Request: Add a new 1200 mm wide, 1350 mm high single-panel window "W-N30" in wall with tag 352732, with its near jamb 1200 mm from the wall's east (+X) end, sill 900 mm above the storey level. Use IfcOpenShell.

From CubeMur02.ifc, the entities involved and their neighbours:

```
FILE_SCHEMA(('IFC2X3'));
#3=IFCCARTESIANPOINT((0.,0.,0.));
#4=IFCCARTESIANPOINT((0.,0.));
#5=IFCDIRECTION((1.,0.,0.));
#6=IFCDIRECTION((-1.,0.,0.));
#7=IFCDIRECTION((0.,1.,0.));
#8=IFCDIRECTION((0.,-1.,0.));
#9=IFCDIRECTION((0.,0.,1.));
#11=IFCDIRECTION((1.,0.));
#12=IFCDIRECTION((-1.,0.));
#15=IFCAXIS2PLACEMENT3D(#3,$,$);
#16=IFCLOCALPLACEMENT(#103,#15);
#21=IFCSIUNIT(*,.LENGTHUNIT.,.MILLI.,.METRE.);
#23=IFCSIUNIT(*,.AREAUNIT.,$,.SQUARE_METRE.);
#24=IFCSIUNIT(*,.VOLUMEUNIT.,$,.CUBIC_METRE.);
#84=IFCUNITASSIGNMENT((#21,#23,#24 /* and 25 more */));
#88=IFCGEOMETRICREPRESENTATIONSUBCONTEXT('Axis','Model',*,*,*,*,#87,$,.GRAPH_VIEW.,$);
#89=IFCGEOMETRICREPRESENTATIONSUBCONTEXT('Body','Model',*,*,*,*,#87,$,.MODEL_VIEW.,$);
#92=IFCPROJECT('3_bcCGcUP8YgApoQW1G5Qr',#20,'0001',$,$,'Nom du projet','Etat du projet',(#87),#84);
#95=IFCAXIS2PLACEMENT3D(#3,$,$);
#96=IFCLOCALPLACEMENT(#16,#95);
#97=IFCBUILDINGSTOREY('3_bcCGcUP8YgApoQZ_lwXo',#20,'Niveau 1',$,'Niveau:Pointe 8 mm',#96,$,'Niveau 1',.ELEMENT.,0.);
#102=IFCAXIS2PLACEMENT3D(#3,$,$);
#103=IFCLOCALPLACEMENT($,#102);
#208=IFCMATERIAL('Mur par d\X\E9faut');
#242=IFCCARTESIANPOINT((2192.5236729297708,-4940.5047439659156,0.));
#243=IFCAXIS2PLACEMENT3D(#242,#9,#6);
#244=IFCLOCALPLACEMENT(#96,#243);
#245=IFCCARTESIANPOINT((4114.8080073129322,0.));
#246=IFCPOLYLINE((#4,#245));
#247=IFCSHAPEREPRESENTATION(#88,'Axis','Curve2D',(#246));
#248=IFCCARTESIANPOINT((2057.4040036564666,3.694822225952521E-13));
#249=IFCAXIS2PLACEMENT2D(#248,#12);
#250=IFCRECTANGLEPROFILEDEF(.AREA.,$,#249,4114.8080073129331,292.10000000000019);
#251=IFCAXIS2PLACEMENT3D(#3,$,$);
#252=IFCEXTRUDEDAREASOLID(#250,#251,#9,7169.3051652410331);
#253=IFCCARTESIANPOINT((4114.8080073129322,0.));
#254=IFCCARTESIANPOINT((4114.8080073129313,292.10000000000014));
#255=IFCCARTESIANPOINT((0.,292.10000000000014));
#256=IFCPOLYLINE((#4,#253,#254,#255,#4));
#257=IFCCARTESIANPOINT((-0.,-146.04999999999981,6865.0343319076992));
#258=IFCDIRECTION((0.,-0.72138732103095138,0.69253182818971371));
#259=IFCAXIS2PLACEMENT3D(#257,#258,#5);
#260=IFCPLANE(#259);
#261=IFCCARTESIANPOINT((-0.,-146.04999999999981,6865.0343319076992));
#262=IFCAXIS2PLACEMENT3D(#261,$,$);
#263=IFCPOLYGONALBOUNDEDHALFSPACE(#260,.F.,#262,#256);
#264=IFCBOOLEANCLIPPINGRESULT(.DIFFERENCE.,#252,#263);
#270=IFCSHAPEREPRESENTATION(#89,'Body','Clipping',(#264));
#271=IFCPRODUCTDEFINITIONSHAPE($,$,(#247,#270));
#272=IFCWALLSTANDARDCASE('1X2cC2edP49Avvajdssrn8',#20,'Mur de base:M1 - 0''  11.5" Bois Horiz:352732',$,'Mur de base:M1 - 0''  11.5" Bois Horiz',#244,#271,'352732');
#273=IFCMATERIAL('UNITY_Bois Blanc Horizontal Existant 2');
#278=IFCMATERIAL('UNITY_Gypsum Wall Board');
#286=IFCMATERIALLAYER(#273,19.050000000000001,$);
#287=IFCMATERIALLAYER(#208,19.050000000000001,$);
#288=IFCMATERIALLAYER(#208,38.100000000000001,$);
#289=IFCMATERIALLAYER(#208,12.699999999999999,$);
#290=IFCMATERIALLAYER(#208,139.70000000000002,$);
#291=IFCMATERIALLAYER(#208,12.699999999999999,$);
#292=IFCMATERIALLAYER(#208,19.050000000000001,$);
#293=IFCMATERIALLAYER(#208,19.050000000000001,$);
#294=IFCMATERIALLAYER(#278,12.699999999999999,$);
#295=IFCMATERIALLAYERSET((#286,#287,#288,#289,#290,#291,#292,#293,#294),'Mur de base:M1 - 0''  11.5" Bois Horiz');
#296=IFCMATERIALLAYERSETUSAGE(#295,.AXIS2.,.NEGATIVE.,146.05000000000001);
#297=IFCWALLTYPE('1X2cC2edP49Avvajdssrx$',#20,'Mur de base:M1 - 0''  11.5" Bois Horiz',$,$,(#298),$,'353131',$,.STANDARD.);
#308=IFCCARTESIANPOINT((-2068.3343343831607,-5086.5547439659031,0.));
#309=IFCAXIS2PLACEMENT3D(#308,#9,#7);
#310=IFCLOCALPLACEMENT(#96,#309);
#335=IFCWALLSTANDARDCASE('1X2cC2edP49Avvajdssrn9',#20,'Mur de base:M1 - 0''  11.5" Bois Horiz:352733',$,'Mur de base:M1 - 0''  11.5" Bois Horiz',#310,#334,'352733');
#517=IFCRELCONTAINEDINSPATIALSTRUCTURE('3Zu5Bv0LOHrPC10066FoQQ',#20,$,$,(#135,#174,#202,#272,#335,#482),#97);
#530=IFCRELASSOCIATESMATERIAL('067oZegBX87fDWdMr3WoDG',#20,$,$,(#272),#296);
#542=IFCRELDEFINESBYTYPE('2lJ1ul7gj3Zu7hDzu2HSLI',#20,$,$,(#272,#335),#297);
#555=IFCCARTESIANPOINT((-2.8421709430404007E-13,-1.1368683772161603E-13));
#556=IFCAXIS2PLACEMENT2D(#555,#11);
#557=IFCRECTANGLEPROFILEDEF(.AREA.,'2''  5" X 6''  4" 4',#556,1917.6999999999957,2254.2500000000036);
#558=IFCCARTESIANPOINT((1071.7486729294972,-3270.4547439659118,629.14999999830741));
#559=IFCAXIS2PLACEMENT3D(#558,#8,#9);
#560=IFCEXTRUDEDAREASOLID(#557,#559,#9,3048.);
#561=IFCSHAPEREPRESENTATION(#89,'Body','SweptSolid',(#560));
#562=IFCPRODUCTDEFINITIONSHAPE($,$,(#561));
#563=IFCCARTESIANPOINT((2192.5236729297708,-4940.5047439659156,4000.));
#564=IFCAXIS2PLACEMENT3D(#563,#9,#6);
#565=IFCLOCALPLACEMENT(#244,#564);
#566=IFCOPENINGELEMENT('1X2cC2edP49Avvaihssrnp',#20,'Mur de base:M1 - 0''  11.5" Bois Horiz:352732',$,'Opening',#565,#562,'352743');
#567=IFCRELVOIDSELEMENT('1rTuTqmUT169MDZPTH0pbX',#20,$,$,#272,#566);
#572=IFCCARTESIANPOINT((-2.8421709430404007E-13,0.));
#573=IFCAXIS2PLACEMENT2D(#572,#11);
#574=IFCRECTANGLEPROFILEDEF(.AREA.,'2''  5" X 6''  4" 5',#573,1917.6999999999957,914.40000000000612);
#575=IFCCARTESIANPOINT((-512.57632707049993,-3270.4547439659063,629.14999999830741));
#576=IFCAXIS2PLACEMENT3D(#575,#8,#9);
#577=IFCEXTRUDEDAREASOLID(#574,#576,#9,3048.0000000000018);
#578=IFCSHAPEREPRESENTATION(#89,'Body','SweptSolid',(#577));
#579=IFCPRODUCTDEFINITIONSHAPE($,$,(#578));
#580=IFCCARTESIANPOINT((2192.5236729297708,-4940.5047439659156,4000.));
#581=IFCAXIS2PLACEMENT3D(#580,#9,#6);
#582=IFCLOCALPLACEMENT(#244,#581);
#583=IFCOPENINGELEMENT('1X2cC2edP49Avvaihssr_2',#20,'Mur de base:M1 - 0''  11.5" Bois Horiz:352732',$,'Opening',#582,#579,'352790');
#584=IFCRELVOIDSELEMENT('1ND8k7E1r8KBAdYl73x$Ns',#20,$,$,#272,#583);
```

```python
import numpy as np
import ifcopenshell
import ifcopenshell.api.feature
import ifcopenshell.api.geometry
import ifcopenshell.api.root
import ifcopenshell.api.spatial
import ifcopenshell.api.type
import ifcopenshell.geom
import ifcopenshell.util.element
import ifcopenshell.util.placement
import ifcopenshell.util.representation
import ifcopenshell.util.shape
import ifcopenshell.util.unit

model = ifcopenshell.open("CubeMur02.ifc")
unit_scale = ifcopenshell.util.unit.calculate_unit_scale(model)
settings = ifcopenshell.geom.settings()


def volume(element):
    """Net volume in cubic metres, openings subtracted."""
    shape = ifcopenshell.geom.create_shape(settings, element)
    return ifcopenshell.util.shape.get_volume(shape.geometry)


wall = model.by_guid("1X2cC2edP49Avvajdssrn8")
storey = ifcopenshell.util.element.get_container(wall, ifc_class="IfcBuildingStorey")
context = ifcopenshell.util.representation.get_context(model, "Model", "Body", "MODEL_VIEW")
before = volume(wall)

width, height, from_end, sill = 1.2, 1.35, 1.2, 0.9  # metres

# The wall runs along its own X axis, and the end named is its -X end.
wall_shape = ifcopenshell.geom.create_shape(settings, wall)
x, y, z = ifcopenshell.util.shape.get_vertices(wall_shape.geometry).T
start = x.min() + from_end
face, thickness = float(y.min()), float(y.max() - y.min())
wall_matrix = ifcopenshell.util.placement.get_local_placement(wall.ObjectPlacement)
level = ifcopenshell.util.placement.get_local_placement(storey.ObjectPlacement)[2, 3]


def in_wall(x, y):
    """Placement at x, y metres in the wall's axes, at sill height."""
    matrix = wall_matrix.copy()
    matrix[:, 3] = wall_matrix @ np.array([x / unit_scale, y / unit_scale, 0.0, 1.0])
    matrix[2, 3] = level + sill / unit_scale
    return matrix


# Opening: a box that overshoots both wall faces by 50 mm.
opening = ifcopenshell.api.root.create_entity(model, ifc_class="IfcOpeningElement")
box = ifcopenshell.api.geometry.add_wall_representation(
    model, context=context, length=width, height=height, thickness=thickness + 0.1
)
ifcopenshell.api.geometry.assign_representation(model, product=opening, representation=box)
ifcopenshell.api.geometry.edit_object_placement(model, product=opening, matrix=in_wall(start, face - 0.05), is_si=False)
ifcopenshell.api.feature.add_feature(model, feature=opening, element=wall)

window = ifcopenshell.api.root.create_entity(model, ifc_class="IfcWindow", name="W-N30")
window.OverallWidth, window.OverallHeight = width / unit_scale, height / unit_scale
body = ifcopenshell.api.geometry.add_window_representation(
    model,
    context=context,
    overall_width=window.OverallWidth,
    overall_height=window.OverallHeight,
    partition_type="SINGLE_PANEL",
)
ifcopenshell.api.geometry.assign_representation(model, product=window, representation=body)
ifcopenshell.api.spatial.assign_container(model, products=[window], relating_structure=storey)
fills = ifcopenshell.api.feature.add_filling(model, opening=opening, element=window)
fills.OwnerHistory = window.OwnerHistory  # required in IFC2X3

# IFC2X3 keeps the operation on the window style.
style = ifcopenshell.api.root.create_entity(model, ifc_class="IfcWindowStyle", name="W-N30")
style.OperationType, style.ConstructionType = "SINGLE_PANEL", "NOTDEFINED"
style.ParameterTakesPrecedence = style.Sizeable = False
ifcopenshell.api.type.assign_type(model, related_objects=[window], relating_type=style)

# Centre the window in the wall's thickness.
ifcopenshell.api.geometry.edit_object_placement(model, product=window, matrix=in_wall(start, face), is_si=False)
window_shape = ifcopenshell.geom.create_shape(settings, window)
depth = ifcopenshell.util.shape.get_vertices(window_shape.geometry)[:, 1]
offset = face + thickness / 2 - (depth.min() + depth.max()) / 2
ifcopenshell.api.geometry.edit_object_placement(model, product=window, matrix=in_wall(start, offset), is_si=False)

after = volume(wall)

print(f"wall volume {before:.3f} -> {after:.3f} m3")

model.write("CubeMur02-out.ifc")
```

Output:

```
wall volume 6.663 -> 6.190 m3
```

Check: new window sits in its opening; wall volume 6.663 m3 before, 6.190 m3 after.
